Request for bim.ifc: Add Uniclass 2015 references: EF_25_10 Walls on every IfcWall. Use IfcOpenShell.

First a look at what the model holds.

```python
import ifcopenshell

model = ifcopenshell.open("bim.ifc")
print(model.schema)
print("classifications:", [c.Name for c in model.by_type("IfcClassification")])
for ifc_class in ("IfcDoor", "IfcRoof", "IfcStair", "IfcWall", "IfcWindow"):
    print(ifc_class, len(model.by_type(ifc_class)))
```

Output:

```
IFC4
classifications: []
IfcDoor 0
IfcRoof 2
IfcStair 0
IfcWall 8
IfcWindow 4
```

```python
import ifcopenshell
import ifcopenshell.api.classification

model = ifcopenshell.open("bim.ifc")

system = ifcopenshell.api.classification.add_classification(model, classification="Uniclass 2015")

codes = {
    "IfcWall": ("EF_25_10", "Walls"),
}
for ifc_class, (code, name) in codes.items():
    products = model.by_type(ifc_class)
    ifcopenshell.api.classification.add_reference(
        model, products=products, classification=system, identification=code, name=name
    )
    print(code, len(products))

model.write("bim_edited.ifc")
```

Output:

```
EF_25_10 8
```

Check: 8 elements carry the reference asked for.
